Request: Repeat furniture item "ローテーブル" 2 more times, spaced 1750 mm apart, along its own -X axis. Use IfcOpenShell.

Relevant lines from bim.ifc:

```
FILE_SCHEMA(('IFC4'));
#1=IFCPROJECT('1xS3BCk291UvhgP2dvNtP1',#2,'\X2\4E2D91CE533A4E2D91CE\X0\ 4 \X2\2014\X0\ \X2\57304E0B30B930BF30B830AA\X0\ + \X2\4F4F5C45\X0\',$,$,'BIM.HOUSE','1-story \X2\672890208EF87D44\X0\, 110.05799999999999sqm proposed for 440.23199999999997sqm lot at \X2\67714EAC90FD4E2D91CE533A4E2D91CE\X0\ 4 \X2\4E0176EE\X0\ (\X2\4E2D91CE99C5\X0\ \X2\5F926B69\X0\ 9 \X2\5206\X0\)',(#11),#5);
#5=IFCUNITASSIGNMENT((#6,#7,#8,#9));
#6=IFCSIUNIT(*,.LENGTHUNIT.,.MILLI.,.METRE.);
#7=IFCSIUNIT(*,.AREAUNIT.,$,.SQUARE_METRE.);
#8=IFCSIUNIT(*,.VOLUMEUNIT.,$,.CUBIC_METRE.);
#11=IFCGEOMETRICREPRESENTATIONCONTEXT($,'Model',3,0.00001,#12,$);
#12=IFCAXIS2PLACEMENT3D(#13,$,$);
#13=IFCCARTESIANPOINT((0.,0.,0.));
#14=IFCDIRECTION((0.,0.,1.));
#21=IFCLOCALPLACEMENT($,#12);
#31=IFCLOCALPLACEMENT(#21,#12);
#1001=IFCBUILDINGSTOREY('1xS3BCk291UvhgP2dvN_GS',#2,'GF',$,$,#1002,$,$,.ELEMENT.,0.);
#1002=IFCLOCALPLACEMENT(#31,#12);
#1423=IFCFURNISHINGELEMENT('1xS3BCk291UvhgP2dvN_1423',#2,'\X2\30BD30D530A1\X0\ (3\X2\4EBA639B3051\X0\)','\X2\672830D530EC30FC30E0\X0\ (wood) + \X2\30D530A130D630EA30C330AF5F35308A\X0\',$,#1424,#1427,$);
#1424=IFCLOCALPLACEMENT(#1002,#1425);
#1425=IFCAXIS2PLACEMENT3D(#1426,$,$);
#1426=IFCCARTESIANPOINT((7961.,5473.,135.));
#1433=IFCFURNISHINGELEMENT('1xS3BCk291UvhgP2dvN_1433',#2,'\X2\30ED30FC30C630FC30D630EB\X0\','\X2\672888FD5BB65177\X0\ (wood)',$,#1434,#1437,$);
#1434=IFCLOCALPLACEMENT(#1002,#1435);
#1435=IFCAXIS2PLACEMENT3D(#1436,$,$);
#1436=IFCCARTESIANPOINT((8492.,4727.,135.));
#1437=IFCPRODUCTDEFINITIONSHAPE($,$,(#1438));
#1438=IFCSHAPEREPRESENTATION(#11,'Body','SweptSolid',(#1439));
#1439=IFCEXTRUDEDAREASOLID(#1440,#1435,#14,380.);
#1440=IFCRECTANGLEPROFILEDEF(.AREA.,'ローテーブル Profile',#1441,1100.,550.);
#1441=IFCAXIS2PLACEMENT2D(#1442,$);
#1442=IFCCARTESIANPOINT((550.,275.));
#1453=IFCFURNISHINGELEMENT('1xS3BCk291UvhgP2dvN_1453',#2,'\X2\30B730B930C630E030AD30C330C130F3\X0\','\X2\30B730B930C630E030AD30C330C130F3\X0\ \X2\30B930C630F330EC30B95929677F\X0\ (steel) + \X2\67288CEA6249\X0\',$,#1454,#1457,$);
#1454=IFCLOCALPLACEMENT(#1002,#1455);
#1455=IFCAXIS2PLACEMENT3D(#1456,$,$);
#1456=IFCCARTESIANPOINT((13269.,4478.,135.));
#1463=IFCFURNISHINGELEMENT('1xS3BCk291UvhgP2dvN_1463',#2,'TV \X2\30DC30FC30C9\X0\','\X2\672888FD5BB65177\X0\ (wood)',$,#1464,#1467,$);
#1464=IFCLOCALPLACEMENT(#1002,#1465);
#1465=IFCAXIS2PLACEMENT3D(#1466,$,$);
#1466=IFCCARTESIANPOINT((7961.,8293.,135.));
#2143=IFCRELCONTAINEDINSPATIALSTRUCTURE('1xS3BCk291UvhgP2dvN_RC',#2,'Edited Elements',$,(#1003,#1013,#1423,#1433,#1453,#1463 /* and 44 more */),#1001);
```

```python
import ifcopenshell
import ifcopenshell.api.geometry
import ifcopenshell.api.root
import ifcopenshell.util.element
import ifcopenshell.util.placement
import ifcopenshell.util.unit

model = ifcopenshell.open("bim.ifc")
unit_scale = ifcopenshell.util.unit.calculate_unit_scale(model)


def reuse_history(source, copy):
    """copy_class also copies each property set's owner history, people and application; keep the originals."""
    for rel in copy.IsDefinedBy:
        if rel.is_a("IfcRelDefinesByProperties") and (history := rel.RelatingPropertyDefinition.OwnerHistory):
            rel.RelatingPropertyDefinition.OwnerHistory = source.OwnerHistory
            ifcopenshell.util.element.remove_deep2(model, history)


source = model.by_id(1433)
base = ifcopenshell.util.placement.get_local_placement(source.ObjectPlacement)
step = -base[:3, 0] * 1.75 / unit_scale

for i in range(1, 3):
    copy = ifcopenshell.api.root.copy_class(model, product=source)
    copy.Representation = ifcopenshell.util.element.copy_deep(
        model, source.Representation, exclude=["IfcGeometricRepresentationContext", "IfcRepresentationMap"]
    )
    reuse_history(source, copy)
    matrix = base.copy()
    matrix[:3, 3] += i * step
    print("added at", matrix[:3, 3].round(3) + 0.0)
    ifcopenshell.api.geometry.edit_object_placement(model, product=copy, matrix=matrix, is_si=False)

model.write("bim_rev.ifc")
```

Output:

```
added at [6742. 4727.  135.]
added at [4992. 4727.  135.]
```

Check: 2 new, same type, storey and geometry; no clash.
